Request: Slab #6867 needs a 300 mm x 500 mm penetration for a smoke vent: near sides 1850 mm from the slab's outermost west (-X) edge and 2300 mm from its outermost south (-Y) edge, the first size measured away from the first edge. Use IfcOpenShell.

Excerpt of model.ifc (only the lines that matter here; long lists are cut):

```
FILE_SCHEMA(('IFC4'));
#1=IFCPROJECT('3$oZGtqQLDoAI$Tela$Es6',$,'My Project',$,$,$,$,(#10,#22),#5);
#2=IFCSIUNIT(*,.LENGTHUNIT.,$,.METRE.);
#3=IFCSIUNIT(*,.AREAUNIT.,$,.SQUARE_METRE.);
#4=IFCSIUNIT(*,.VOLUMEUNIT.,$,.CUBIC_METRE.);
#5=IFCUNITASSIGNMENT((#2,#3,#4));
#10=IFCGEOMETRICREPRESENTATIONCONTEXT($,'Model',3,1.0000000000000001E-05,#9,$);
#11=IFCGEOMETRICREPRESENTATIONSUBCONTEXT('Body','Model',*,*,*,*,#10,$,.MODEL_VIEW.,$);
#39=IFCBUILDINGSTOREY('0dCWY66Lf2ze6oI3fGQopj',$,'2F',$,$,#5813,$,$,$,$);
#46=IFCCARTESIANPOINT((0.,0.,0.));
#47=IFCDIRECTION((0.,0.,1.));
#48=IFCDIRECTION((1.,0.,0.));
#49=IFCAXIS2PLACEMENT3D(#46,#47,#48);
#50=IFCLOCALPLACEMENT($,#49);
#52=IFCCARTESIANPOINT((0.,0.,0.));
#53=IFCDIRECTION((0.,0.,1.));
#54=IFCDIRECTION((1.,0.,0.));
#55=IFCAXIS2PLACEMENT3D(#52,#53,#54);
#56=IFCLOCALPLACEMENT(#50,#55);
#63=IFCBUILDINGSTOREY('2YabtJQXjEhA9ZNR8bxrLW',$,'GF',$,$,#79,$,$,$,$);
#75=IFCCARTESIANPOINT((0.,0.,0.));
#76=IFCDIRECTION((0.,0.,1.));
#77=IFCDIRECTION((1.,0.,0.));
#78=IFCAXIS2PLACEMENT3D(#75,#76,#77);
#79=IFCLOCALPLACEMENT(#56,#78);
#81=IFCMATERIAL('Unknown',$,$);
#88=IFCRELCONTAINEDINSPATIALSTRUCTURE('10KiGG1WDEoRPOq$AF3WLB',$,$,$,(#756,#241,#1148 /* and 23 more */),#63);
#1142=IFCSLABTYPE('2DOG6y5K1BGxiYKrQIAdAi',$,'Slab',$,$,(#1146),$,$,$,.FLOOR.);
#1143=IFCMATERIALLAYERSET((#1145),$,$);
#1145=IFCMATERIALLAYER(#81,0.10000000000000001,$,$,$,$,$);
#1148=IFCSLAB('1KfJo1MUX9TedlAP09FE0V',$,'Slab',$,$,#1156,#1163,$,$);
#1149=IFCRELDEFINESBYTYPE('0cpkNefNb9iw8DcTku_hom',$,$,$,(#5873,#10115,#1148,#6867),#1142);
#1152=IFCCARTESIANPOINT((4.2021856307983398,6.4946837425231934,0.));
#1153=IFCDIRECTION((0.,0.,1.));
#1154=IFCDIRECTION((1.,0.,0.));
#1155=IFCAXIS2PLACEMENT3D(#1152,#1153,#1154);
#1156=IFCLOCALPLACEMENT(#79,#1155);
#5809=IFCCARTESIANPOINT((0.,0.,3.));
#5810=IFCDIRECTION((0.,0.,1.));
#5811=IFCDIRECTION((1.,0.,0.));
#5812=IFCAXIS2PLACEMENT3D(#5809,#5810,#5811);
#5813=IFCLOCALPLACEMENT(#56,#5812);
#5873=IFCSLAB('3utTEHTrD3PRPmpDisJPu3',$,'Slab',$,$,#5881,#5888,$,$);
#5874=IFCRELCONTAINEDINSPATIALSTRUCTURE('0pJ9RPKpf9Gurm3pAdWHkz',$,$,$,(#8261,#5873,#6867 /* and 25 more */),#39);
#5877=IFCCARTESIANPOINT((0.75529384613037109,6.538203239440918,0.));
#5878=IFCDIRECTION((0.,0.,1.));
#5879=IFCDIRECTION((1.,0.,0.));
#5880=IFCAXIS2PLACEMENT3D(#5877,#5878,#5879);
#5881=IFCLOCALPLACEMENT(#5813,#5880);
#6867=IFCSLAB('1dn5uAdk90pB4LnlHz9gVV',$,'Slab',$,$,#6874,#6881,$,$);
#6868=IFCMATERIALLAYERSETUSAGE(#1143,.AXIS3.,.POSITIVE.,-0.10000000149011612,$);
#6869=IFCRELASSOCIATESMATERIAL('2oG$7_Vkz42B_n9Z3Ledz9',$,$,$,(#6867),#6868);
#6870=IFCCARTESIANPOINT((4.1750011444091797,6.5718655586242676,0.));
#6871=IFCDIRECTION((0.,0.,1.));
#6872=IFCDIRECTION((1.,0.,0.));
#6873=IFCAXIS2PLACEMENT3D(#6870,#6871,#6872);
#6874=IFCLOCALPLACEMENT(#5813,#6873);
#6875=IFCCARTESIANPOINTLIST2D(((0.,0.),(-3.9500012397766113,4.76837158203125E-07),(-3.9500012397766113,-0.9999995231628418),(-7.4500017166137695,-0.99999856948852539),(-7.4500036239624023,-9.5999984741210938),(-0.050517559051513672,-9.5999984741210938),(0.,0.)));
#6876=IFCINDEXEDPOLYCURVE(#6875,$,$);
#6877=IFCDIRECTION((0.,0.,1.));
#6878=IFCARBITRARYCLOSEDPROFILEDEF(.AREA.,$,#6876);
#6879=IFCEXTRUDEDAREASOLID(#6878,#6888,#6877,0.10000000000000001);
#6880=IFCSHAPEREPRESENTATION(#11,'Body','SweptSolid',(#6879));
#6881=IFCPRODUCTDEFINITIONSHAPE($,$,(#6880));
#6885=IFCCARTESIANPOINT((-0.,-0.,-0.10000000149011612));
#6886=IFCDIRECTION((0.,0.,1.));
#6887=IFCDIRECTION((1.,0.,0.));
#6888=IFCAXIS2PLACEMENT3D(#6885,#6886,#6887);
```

```python
import numpy as np
import ifcopenshell
import ifcopenshell.api.feature
import ifcopenshell.api.geometry
import ifcopenshell.api.root
import ifcopenshell.geom
import ifcopenshell.util.placement
import ifcopenshell.util.representation
import ifcopenshell.util.shape
import ifcopenshell.util.unit

model = ifcopenshell.open("model.ifc")
unit_scale = ifcopenshell.util.unit.calculate_unit_scale(model)
settings = ifcopenshell.geom.settings()


def volume(element):
    """Net volume in cubic metres, openings subtracted."""
    shape = ifcopenshell.geom.create_shape(settings, element)
    return ifcopenshell.util.shape.get_volume(shape.geometry)


slab = model.by_id(6867)
before = volume(slab)

# Extent in the slab's own axes, in metres. The edges named are its -X and -Y sides.
slab_shape = ifcopenshell.geom.create_shape(settings, slab)
vertices = ifcopenshell.util.shape.get_vertices(slab_shape.geometry)
x_min, y_min, bottom = vertices.min(axis=0)
top = vertices[:, 2].max()

opening = ifcopenshell.api.root.create_entity(model, ifc_class="IfcOpeningElement", name="Smoke vent opening", predefined_type="OPENING")
context = ifcopenshell.util.representation.get_context(model, "Model", "Body", "MODEL_VIEW")
width, depth = 0.3, 0.5
outline = [(0.0, 0.0), (width, 0.0), (width, depth), (0.0, depth), (0.0, 0.0)]
# Overshoot both faces by 50 mm so the cut is clean.
shape = ifcopenshell.api.geometry.add_slab_representation(
    model, context=context, depth=top - bottom + 0.1, polyline=outline
)
ifcopenshell.api.geometry.assign_representation(model, product=opening, representation=shape)

matrix = ifcopenshell.util.placement.get_local_placement(slab.ObjectPlacement)
matrix[:, 3] = matrix @ np.append(np.array([x_min + 1.85, y_min + 2.3, bottom - 0.05]) / unit_scale, 1.0)
ifcopenshell.api.geometry.edit_object_placement(model, product=opening, matrix=matrix, is_si=False)
ifcopenshell.api.feature.add_feature(model, feature=opening, element=slab)

after = volume(slab)

print(f"slab volume {before:.3f} -> {after:.3f} m3")

model.write("model_v2.ifc")
```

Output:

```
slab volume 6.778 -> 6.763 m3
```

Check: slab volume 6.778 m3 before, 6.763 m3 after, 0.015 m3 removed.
